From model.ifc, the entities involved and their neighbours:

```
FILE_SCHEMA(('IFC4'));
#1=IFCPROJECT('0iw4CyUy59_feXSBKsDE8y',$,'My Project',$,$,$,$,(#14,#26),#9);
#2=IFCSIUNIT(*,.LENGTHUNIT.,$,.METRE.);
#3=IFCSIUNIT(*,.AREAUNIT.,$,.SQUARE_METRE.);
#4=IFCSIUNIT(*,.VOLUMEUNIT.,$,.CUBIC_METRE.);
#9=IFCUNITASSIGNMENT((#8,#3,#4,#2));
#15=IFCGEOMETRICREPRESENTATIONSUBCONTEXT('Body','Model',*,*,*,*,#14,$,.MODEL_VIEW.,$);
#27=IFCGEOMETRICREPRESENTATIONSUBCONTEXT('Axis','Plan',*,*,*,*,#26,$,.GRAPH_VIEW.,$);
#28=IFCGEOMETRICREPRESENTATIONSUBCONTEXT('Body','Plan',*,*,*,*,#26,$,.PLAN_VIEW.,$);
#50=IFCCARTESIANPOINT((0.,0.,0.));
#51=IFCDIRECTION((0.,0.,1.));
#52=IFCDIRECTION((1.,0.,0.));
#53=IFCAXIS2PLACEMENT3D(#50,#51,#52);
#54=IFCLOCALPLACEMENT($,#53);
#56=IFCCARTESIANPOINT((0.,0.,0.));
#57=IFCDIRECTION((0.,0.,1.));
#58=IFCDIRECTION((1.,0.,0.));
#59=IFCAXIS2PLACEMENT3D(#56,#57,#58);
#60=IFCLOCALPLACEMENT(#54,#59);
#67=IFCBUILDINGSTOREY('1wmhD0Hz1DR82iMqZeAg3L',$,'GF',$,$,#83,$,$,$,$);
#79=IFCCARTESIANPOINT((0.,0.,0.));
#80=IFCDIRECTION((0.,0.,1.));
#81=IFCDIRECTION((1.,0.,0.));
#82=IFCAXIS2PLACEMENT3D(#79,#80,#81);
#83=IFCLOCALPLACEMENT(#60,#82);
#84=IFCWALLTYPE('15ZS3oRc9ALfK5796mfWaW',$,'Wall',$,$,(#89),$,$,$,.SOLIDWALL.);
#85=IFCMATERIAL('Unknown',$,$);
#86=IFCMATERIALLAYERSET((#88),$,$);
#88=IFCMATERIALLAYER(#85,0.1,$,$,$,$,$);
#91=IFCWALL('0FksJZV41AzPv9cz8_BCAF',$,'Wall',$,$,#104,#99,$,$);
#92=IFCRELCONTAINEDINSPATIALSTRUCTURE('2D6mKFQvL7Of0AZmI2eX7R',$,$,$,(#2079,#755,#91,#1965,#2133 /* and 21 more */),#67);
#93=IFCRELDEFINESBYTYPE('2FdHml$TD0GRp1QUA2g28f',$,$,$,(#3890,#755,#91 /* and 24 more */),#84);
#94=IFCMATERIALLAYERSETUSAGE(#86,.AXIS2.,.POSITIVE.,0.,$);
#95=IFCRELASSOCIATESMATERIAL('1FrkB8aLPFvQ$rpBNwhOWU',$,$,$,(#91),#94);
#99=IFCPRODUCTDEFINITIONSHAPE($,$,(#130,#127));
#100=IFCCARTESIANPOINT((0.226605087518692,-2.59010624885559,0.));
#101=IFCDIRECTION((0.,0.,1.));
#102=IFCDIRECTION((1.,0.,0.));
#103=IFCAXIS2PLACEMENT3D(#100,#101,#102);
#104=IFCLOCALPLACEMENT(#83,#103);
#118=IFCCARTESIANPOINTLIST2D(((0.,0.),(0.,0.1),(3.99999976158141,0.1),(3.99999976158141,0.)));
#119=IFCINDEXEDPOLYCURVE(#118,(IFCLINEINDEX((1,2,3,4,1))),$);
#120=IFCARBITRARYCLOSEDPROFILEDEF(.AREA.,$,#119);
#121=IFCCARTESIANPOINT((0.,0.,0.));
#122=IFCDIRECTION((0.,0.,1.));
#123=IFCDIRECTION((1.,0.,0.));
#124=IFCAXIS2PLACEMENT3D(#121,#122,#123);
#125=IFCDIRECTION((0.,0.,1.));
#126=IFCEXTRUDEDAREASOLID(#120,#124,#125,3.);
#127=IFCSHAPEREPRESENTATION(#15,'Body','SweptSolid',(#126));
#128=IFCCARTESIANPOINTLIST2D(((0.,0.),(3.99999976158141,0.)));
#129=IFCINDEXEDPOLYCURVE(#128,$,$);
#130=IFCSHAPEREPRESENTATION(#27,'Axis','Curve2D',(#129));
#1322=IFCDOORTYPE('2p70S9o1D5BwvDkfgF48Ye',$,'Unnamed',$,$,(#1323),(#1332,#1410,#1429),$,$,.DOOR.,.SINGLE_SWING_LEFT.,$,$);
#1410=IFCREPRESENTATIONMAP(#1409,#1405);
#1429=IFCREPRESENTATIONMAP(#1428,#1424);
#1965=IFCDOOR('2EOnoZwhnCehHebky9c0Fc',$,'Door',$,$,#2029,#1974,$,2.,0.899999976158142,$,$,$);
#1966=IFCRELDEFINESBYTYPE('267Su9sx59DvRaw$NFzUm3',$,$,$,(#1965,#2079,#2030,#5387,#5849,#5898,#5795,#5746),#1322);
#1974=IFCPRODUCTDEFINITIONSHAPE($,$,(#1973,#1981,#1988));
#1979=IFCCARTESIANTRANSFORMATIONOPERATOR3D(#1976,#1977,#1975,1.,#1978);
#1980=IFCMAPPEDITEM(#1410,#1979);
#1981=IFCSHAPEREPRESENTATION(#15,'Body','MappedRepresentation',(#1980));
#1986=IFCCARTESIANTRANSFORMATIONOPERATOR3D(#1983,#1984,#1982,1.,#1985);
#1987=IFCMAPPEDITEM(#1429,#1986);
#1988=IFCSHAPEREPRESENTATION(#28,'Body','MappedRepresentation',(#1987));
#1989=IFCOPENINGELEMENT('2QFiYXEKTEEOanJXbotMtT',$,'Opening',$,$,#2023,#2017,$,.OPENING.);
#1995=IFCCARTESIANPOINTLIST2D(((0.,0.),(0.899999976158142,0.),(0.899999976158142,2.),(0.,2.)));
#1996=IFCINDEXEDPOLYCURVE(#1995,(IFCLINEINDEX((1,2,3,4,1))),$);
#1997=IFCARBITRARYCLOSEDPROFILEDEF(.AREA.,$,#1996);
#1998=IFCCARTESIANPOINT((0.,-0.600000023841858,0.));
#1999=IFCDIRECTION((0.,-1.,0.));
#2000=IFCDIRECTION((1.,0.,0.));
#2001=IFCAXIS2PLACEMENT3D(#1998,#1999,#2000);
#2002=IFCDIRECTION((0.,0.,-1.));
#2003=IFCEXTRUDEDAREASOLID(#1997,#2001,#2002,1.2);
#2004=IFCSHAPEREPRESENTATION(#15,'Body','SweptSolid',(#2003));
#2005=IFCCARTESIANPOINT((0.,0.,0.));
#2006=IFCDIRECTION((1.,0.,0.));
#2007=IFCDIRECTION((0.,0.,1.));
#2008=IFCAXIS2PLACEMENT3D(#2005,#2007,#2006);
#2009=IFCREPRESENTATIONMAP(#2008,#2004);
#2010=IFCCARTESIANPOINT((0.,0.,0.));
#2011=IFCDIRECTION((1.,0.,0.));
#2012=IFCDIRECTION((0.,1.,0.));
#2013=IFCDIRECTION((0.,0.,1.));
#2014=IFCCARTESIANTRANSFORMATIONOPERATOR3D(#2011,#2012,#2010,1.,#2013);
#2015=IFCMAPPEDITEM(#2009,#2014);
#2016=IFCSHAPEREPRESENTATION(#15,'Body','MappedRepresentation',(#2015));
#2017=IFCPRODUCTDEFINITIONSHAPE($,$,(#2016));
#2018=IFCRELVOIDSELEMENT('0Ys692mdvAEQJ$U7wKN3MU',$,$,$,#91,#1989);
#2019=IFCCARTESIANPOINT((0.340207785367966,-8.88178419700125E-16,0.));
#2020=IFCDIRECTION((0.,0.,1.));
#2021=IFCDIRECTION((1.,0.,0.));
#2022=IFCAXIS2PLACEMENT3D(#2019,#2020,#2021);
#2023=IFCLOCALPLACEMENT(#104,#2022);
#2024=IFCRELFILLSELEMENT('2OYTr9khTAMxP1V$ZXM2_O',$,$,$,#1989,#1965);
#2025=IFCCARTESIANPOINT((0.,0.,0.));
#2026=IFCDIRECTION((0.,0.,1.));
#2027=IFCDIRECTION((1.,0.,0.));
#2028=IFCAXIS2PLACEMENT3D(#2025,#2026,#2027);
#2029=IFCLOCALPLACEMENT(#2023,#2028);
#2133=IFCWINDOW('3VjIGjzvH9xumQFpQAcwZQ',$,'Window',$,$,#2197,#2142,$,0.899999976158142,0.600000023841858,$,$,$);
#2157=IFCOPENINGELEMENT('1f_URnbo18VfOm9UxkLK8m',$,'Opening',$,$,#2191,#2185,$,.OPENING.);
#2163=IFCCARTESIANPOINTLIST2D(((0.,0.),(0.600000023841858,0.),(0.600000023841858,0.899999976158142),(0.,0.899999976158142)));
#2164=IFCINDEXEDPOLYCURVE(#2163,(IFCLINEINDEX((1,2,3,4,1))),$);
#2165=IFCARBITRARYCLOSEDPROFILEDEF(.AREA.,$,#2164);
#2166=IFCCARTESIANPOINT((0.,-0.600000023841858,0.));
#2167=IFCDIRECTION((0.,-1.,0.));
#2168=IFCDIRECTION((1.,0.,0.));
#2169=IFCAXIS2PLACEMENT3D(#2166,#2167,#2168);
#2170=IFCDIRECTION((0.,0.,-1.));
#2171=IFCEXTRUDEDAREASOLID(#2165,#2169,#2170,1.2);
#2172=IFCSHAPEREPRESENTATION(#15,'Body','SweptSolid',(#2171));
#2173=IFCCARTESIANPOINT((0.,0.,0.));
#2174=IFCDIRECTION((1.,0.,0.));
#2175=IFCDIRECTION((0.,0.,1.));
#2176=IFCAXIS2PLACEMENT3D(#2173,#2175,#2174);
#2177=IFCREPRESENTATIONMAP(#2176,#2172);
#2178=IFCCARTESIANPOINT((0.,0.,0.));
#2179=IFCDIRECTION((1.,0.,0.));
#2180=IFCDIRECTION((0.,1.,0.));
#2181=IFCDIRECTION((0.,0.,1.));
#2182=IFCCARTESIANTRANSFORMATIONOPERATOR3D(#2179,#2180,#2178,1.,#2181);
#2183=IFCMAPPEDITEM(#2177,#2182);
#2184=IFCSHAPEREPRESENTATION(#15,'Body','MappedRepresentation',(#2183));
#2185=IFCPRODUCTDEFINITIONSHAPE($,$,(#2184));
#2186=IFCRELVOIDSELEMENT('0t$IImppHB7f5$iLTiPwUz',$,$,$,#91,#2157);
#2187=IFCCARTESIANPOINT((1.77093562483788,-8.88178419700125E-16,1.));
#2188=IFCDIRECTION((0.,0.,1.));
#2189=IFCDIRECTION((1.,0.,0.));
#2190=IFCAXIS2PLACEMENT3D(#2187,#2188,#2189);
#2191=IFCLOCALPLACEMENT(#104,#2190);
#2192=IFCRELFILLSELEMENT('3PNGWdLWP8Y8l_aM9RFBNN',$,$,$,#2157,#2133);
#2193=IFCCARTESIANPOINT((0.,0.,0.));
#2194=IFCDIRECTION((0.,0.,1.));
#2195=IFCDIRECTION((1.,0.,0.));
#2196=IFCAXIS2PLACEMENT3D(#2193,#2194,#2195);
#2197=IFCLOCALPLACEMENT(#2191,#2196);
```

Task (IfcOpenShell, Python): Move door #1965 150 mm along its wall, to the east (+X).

```python
import ifcopenshell
import ifcopenshell.api.geometry
import ifcopenshell.util.placement

model = ifcopenshell.open("model.ifc")

door = model.by_guid("2EOnoZwhnCehHebky9c0Fc")
opening = door.FillsVoids[0].RelatingOpeningElement
wall = opening.VoidsElements[0].RelatingBuildingElement

wall_matrix = ifcopenshell.util.placement.get_local_placement(wall.ObjectPlacement)
shift = wall_matrix[:3, 0] * 0.15
before = ifcopenshell.util.placement.get_local_placement(door.ObjectPlacement)[:3, 3].copy()

# The door is placed relative to its opening, so it follows when the opening moves.
matrix = ifcopenshell.util.placement.get_local_placement(opening.ObjectPlacement)
matrix[:3, 3] += shift
ifcopenshell.api.geometry.edit_object_placement(
    model, product=opening, matrix=matrix, is_si=False, should_transform_children=True
)

after = ifcopenshell.util.placement.get_local_placement(door.ObjectPlacement)[:3, 3]
print("door moved by", (after - before).round(3) + 0.0)

model.write("model_updated.ifc")
```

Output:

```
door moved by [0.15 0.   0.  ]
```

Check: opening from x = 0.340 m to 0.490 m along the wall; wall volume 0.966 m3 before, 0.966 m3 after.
